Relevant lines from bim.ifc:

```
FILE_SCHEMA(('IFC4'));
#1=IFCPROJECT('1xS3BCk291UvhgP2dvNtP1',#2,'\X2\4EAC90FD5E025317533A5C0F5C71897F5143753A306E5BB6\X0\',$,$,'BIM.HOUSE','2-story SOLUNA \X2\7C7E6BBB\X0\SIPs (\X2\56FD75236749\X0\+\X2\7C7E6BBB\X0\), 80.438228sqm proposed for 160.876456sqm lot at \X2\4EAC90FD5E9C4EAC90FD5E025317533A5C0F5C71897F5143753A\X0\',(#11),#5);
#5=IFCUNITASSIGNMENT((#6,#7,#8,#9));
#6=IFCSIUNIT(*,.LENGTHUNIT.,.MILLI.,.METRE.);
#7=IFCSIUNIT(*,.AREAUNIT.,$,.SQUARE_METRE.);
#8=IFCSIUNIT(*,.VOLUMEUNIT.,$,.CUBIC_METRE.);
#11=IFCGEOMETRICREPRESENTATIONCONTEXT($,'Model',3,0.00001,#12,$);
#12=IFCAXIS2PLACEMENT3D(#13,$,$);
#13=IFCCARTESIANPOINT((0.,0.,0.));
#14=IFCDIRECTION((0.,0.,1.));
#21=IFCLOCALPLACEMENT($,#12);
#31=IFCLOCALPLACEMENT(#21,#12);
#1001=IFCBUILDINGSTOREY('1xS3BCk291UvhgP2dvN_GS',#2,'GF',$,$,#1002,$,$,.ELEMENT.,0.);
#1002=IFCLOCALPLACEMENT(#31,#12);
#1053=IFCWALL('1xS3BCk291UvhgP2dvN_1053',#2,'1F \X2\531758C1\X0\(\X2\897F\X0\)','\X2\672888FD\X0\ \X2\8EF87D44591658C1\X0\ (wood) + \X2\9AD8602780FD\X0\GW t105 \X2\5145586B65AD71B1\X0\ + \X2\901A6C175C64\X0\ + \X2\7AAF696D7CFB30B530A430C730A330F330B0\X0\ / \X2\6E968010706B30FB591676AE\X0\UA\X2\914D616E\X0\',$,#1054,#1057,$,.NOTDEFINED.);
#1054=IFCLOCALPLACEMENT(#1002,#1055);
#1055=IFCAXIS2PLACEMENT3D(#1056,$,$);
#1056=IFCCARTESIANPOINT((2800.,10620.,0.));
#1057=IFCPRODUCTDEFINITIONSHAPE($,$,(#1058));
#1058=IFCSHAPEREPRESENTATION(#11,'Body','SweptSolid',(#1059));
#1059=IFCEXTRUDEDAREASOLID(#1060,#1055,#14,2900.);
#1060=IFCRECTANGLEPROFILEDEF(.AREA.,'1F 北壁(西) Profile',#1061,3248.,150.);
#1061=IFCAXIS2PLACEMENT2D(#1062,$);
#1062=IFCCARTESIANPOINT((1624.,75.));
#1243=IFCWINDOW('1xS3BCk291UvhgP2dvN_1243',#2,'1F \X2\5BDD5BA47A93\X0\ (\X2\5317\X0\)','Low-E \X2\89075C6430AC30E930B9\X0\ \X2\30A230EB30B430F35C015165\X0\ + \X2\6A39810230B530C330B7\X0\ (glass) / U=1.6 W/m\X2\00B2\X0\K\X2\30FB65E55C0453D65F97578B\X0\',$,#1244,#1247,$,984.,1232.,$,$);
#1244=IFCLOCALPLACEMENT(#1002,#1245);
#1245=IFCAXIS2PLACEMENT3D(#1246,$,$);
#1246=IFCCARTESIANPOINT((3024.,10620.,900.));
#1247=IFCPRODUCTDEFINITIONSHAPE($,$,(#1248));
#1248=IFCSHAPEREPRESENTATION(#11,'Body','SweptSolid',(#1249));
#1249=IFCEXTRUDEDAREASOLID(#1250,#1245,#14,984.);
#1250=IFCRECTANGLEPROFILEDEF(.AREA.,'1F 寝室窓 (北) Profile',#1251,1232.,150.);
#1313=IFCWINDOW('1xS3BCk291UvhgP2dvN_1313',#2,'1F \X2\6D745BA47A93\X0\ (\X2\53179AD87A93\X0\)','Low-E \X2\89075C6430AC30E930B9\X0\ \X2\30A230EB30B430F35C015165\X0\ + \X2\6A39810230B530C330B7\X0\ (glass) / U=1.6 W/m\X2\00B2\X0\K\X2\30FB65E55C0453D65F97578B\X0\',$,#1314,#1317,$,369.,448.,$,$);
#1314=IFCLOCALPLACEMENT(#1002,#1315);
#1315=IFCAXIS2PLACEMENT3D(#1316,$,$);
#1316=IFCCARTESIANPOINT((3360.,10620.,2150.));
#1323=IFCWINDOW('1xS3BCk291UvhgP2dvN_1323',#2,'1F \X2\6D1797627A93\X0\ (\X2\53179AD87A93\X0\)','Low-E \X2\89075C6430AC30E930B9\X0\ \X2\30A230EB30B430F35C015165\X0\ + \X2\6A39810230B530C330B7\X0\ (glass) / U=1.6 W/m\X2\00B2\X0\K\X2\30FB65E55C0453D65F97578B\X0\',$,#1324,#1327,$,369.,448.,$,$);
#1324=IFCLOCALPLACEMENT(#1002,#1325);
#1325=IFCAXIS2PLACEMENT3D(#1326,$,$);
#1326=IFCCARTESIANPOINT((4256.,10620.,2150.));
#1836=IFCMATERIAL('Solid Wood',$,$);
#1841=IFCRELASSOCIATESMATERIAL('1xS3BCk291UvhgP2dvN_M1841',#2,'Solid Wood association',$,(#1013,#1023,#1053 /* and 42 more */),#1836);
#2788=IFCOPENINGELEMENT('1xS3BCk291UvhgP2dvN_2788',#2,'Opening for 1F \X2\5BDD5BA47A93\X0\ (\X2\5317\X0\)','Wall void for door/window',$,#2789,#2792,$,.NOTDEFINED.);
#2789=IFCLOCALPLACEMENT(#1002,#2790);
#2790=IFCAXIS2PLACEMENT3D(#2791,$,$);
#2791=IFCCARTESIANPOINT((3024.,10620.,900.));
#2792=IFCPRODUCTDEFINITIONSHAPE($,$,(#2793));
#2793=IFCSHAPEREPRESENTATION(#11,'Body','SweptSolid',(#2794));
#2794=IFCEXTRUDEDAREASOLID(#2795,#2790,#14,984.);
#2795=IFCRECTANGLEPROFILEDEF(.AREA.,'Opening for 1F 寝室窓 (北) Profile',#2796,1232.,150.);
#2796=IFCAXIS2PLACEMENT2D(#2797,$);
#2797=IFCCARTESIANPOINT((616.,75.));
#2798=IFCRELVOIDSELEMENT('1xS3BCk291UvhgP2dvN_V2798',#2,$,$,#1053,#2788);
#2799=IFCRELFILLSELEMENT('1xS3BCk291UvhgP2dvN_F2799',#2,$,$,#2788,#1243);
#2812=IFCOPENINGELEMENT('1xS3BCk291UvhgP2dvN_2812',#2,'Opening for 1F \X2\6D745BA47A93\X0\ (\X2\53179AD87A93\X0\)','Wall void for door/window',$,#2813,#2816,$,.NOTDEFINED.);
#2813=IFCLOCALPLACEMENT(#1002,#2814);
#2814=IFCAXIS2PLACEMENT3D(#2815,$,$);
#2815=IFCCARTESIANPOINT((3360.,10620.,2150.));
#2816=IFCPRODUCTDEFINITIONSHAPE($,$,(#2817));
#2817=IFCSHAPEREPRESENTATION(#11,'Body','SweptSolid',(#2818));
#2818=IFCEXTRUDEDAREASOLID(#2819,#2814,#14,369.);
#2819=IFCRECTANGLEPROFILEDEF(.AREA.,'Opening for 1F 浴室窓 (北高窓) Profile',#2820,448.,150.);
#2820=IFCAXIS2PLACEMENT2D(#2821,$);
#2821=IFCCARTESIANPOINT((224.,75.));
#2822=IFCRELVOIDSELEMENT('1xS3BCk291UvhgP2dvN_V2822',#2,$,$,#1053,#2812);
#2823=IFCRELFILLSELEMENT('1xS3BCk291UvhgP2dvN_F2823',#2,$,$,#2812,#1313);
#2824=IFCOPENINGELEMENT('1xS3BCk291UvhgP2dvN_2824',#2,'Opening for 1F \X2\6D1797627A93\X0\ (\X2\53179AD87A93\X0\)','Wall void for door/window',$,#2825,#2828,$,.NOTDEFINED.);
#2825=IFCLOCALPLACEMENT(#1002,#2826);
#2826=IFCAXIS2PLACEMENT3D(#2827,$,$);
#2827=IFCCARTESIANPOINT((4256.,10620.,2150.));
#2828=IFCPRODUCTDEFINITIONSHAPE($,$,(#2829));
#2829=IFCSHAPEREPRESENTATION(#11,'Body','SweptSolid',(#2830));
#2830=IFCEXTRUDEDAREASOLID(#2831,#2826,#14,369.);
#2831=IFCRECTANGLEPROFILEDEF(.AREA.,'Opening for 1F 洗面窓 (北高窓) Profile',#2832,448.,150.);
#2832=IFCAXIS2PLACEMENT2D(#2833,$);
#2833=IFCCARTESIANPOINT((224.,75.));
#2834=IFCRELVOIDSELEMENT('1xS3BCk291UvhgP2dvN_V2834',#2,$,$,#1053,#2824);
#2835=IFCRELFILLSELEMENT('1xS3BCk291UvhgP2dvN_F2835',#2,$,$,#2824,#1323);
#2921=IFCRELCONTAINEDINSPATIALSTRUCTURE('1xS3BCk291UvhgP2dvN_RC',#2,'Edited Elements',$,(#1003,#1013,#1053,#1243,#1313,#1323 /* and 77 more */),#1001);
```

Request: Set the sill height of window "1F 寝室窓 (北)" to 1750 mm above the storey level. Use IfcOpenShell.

```python
import numpy as np
import ifcopenshell
import ifcopenshell.api.geometry
import ifcopenshell.geom
import ifcopenshell.util.element
import ifcopenshell.util.placement
import ifcopenshell.util.shape
import ifcopenshell.util.unit

model = ifcopenshell.open("bim.ifc")
unit_scale = ifcopenshell.util.unit.calculate_unit_scale(model)

window = model.by_guid("1xS3BCk291UvhgP2dvN_1243")
opening = window.FillsVoids[0].RelatingOpeningElement
storey = ifcopenshell.util.element.get_container(window, ifc_class="IfcBuildingStorey")
level = ifcopenshell.util.placement.get_local_placement(storey.ObjectPlacement)[2, 3]

# The opening's origin need not be at the sill, so measure its lowest point.
shape = ifcopenshell.geom.create_shape(ifcopenshell.geom.settings(), opening)
bottom = ifcopenshell.util.shape.get_shape_bottom_elevation(shape, shape.geometry) / unit_scale
dz = level + 1750.0 - bottom

shift = np.array([0.0, 0.0, dz])
# The window is not placed relative to its opening, so move both.
for product in (opening, window):
    matrix = ifcopenshell.util.placement.get_local_placement(product.ObjectPlacement)
    matrix[:3, 3] += shift
    ifcopenshell.api.geometry.edit_object_placement(model, product=product, matrix=matrix, is_si=False)

print(f"moved by {dz * unit_scale:+.3f} m")

model.write("bim-out.ifc")
```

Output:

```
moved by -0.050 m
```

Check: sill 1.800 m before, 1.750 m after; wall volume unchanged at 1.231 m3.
